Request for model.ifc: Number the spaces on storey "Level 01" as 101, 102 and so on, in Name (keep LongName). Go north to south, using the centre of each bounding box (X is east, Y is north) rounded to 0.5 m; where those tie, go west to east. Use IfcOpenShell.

First a look at what the model holds.

```python
import ifcopenshell
import ifcopenshell.util.element
import ifcopenshell.util.placement

model = ifcopenshell.open("model.ifc")
print(model.schema)
storey = next(s for s in model.by_type("IfcBuildingStorey") if s.Name == "Level 01")
spaces = [e for e in ifcopenshell.util.element.get_decomposition(storey) if e.is_a("IfcSpace")]
for e in sorted(spaces, key=lambda e: e.id()):
    origin = ifcopenshell.util.placement.get_local_placement(e.ObjectPlacement)[:3, 3]
    print(e.id(), e.Name, e.LongName, origin.round(2) + 0.0, sep=" | ")
```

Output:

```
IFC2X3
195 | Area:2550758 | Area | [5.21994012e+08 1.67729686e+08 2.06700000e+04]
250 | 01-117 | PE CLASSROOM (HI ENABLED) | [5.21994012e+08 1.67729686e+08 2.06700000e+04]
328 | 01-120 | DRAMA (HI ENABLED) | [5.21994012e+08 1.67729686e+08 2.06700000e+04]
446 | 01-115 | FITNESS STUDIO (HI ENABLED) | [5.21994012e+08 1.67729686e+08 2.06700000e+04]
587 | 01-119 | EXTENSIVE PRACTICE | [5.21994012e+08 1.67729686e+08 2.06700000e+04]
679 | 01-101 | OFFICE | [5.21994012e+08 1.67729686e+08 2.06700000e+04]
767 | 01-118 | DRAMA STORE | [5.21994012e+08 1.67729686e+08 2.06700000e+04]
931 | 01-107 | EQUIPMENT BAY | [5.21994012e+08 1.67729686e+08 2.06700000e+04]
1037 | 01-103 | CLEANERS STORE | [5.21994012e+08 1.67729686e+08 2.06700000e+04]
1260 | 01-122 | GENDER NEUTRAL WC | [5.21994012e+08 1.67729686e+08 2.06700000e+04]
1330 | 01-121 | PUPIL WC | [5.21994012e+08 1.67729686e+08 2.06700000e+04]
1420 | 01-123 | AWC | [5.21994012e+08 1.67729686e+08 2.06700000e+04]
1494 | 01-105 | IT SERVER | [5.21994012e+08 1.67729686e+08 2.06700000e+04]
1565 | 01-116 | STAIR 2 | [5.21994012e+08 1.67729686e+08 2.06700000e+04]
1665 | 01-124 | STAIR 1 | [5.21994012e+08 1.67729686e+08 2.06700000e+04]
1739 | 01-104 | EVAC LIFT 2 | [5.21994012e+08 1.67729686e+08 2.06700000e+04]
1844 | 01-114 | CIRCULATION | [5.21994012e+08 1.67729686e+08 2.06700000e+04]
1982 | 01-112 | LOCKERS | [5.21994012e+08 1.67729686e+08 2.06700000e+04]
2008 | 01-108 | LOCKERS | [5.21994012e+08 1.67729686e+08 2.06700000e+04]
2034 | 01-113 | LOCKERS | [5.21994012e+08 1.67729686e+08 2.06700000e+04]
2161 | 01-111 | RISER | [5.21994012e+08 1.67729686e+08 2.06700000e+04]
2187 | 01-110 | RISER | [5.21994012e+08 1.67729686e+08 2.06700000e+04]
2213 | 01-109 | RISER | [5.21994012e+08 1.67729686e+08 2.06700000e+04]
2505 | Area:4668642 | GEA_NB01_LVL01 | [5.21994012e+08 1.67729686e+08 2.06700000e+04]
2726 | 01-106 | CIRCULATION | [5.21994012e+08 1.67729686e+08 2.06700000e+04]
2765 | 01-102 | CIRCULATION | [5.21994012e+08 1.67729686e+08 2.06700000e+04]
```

```python
import ifcopenshell
import ifcopenshell.geom
import ifcopenshell.util.element
import ifcopenshell.util.shape

model = ifcopenshell.open("model.ifc")
settings = ifcopenshell.geom.settings()
settings.set("use-world-coords", True)


def centre(element):
    shape = ifcopenshell.geom.create_shape(settings, element)
    return ifcopenshell.util.shape.get_bbox_centroid(shape.geometry)


storey = next(s for s in model.by_type("IfcBuildingStorey") if s.Name == "Level 01")
spaces = [e for e in ifcopenshell.util.element.get_decomposition(storey) if e.is_a("IfcSpace")]

# Insertion points can sit at a corner or the storey origin, so sort by the geometry (in metres).
centres = {e: centre(e) for e in spaces}
spaces.sort(key=lambda e: (-round(centres[e][1] / 0.5), centres[e][0]))

for i, e in enumerate(spaces, start=1):
    number = f"1{i:02d}"
    e.Name = number
    print(e.id(), number)

model.write("model_v2.ifc")
```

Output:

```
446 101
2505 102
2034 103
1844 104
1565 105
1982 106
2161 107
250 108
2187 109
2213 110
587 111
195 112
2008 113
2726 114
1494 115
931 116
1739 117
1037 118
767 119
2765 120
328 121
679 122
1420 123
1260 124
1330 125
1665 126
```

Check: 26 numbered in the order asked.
